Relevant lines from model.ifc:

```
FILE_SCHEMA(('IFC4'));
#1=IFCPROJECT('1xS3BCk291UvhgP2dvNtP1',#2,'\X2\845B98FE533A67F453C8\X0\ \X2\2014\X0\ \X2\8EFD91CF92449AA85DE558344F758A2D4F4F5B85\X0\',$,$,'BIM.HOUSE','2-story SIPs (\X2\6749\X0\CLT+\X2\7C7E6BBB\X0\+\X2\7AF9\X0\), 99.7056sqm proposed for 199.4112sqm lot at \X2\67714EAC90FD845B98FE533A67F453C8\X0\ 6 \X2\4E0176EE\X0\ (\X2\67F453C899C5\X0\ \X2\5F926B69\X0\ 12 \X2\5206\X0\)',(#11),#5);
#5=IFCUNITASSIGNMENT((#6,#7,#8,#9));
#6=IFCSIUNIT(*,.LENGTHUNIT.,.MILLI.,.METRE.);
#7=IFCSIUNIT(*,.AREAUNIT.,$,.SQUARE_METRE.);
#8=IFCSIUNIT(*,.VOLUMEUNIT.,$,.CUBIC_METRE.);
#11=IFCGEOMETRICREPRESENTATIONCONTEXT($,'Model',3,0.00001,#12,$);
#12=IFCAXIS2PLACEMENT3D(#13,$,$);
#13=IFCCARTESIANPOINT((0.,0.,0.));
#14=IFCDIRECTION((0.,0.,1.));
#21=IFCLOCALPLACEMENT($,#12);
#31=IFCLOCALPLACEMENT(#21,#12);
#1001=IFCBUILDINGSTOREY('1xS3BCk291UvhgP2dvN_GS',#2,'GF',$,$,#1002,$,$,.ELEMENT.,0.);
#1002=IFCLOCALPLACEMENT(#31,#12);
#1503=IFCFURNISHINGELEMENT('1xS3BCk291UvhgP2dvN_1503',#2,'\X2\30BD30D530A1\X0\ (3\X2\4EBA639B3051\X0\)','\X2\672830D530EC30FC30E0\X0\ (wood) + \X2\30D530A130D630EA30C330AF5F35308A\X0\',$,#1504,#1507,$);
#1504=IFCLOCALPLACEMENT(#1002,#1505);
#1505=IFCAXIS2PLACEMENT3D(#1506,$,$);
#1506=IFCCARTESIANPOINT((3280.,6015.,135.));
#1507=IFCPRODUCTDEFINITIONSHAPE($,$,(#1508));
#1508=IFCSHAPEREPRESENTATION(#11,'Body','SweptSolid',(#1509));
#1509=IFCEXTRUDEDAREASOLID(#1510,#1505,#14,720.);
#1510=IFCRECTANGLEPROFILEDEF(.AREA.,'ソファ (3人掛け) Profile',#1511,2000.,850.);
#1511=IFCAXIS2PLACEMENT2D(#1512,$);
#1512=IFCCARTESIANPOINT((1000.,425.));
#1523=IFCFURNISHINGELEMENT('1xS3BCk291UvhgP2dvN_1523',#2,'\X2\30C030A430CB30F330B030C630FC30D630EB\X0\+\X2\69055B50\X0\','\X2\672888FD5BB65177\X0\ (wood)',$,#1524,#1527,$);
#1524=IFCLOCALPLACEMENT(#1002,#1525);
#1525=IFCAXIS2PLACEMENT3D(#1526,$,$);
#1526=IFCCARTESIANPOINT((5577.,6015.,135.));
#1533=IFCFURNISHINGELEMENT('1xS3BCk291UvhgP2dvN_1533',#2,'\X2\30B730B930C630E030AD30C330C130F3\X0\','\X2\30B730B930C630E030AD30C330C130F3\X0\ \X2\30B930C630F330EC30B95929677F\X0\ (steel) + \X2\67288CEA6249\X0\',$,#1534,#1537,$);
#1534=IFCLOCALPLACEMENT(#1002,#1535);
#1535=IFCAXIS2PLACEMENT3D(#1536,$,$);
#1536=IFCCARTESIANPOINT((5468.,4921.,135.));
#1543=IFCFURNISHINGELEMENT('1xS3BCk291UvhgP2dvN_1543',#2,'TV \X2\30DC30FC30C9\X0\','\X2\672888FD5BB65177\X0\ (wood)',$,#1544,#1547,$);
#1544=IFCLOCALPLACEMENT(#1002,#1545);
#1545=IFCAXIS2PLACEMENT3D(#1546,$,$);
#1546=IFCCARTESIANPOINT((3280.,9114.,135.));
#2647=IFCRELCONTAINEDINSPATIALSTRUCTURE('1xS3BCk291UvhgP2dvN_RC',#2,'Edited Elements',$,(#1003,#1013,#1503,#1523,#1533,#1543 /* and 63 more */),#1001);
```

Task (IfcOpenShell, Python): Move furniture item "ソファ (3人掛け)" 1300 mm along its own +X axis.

```python
import ifcopenshell
import ifcopenshell.api.geometry
import ifcopenshell.util.placement

model = ifcopenshell.open("model.ifc")

item = model.by_guid("1xS3BCk291UvhgP2dvN_1503")
matrix = ifcopenshell.util.placement.get_local_placement(item.ObjectPlacement)
matrix[:3, 3] += matrix[:3, 0] * 1300.0
ifcopenshell.api.geometry.edit_object_placement(model, product=item, matrix=matrix, is_si=False)

print(ifcopenshell.util.placement.get_local_placement(item.ObjectPlacement).round(3) + 0.0)

model.write("model_updated.ifc")
```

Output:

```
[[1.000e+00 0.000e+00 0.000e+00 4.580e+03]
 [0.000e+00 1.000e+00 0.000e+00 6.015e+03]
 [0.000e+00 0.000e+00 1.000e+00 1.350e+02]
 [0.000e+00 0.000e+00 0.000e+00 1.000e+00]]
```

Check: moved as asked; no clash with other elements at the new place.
